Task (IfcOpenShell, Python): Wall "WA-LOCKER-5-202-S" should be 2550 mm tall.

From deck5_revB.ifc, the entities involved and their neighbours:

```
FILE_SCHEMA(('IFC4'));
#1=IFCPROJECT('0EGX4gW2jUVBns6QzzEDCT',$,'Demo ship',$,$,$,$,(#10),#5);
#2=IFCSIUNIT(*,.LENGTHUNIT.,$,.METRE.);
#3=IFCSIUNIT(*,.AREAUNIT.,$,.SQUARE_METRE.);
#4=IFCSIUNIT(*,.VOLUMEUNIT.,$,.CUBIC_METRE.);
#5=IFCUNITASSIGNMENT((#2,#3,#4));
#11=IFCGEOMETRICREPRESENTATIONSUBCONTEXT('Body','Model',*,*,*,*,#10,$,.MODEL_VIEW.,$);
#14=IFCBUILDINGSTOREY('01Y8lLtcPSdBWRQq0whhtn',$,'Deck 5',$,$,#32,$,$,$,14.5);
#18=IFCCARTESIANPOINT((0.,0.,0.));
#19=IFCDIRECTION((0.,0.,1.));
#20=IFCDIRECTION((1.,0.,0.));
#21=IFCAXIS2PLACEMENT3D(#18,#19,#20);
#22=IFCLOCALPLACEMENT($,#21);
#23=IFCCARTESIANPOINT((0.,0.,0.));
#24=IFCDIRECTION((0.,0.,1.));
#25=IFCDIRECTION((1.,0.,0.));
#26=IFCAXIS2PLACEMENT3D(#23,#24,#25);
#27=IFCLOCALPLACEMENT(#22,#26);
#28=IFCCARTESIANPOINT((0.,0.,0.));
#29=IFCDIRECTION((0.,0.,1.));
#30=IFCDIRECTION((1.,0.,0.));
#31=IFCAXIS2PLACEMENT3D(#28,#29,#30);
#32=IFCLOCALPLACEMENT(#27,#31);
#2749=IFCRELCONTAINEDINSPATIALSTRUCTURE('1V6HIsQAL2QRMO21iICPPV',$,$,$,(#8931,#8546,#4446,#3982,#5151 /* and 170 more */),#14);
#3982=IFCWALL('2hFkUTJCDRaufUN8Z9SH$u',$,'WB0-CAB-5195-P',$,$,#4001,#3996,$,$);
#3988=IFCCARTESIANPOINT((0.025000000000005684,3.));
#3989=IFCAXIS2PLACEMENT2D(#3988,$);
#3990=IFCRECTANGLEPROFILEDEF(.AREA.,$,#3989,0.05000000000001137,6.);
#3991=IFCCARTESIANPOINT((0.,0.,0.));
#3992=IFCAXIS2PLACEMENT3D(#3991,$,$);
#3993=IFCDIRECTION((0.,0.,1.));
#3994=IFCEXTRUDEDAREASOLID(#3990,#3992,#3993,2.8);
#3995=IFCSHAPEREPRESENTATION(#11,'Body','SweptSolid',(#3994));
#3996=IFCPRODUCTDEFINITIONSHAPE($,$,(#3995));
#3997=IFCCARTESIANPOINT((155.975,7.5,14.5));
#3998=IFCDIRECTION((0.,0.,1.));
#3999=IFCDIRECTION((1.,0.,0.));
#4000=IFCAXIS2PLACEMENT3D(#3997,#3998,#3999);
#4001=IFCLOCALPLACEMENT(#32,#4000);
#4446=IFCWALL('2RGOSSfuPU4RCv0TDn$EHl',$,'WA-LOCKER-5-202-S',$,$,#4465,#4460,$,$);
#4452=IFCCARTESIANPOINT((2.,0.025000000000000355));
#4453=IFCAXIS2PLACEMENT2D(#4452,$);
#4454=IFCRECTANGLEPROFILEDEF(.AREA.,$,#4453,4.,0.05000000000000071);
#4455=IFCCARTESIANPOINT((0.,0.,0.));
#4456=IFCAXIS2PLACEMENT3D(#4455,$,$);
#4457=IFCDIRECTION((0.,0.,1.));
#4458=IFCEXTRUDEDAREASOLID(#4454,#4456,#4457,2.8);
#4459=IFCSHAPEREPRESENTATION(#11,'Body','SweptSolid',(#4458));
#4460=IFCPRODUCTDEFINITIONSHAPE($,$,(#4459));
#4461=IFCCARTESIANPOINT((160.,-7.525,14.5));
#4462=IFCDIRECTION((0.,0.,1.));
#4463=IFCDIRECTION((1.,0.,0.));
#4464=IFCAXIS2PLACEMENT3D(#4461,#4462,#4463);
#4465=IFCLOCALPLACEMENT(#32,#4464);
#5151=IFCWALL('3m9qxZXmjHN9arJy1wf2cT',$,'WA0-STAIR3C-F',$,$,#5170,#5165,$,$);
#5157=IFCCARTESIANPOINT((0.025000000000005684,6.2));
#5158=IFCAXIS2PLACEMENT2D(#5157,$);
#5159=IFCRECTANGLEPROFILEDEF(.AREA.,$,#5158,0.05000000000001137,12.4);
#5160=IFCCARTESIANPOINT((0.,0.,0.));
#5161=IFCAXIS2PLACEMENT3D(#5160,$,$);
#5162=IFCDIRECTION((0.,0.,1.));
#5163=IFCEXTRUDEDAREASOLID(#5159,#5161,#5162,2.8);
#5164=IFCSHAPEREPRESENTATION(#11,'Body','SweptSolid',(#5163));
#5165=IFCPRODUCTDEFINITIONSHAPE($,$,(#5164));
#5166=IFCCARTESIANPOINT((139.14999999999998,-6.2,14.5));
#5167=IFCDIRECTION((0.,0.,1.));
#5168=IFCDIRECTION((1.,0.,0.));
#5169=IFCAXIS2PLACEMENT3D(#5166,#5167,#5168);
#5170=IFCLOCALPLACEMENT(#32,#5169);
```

```python
import ifcopenshell
import ifcopenshell.geom
import ifcopenshell.util.representation
import ifcopenshell.util.shape
import ifcopenshell.util.unit

model = ifcopenshell.open("deck5_revB.ifc")
unit_scale = ifcopenshell.util.unit.calculate_unit_scale(model)
settings = ifcopenshell.geom.settings()


def volume(element):
    """Net volume in cubic metres, openings subtracted."""
    shape = ifcopenshell.geom.create_shape(settings, element)
    return ifcopenshell.util.shape.get_volume(shape.geometry)


wall = model.by_guid("2RGOSSfuPU4RCv0TDn$EHl")
before = volume(wall)

body = ifcopenshell.util.representation.get_representation(wall, "Model", "Body")
solid = body.Items[0]
old_height = solid.Depth
solid.Depth = 2.55 / unit_scale
after = volume(wall)

print(f"height {old_height:g} -> {solid.Depth:g}, volume {before:.3f} -> {after:.3f} m3")

model.write("deck5_revB_v2.ifc")
```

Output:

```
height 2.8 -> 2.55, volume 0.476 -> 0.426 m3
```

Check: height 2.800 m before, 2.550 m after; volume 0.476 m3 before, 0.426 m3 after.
